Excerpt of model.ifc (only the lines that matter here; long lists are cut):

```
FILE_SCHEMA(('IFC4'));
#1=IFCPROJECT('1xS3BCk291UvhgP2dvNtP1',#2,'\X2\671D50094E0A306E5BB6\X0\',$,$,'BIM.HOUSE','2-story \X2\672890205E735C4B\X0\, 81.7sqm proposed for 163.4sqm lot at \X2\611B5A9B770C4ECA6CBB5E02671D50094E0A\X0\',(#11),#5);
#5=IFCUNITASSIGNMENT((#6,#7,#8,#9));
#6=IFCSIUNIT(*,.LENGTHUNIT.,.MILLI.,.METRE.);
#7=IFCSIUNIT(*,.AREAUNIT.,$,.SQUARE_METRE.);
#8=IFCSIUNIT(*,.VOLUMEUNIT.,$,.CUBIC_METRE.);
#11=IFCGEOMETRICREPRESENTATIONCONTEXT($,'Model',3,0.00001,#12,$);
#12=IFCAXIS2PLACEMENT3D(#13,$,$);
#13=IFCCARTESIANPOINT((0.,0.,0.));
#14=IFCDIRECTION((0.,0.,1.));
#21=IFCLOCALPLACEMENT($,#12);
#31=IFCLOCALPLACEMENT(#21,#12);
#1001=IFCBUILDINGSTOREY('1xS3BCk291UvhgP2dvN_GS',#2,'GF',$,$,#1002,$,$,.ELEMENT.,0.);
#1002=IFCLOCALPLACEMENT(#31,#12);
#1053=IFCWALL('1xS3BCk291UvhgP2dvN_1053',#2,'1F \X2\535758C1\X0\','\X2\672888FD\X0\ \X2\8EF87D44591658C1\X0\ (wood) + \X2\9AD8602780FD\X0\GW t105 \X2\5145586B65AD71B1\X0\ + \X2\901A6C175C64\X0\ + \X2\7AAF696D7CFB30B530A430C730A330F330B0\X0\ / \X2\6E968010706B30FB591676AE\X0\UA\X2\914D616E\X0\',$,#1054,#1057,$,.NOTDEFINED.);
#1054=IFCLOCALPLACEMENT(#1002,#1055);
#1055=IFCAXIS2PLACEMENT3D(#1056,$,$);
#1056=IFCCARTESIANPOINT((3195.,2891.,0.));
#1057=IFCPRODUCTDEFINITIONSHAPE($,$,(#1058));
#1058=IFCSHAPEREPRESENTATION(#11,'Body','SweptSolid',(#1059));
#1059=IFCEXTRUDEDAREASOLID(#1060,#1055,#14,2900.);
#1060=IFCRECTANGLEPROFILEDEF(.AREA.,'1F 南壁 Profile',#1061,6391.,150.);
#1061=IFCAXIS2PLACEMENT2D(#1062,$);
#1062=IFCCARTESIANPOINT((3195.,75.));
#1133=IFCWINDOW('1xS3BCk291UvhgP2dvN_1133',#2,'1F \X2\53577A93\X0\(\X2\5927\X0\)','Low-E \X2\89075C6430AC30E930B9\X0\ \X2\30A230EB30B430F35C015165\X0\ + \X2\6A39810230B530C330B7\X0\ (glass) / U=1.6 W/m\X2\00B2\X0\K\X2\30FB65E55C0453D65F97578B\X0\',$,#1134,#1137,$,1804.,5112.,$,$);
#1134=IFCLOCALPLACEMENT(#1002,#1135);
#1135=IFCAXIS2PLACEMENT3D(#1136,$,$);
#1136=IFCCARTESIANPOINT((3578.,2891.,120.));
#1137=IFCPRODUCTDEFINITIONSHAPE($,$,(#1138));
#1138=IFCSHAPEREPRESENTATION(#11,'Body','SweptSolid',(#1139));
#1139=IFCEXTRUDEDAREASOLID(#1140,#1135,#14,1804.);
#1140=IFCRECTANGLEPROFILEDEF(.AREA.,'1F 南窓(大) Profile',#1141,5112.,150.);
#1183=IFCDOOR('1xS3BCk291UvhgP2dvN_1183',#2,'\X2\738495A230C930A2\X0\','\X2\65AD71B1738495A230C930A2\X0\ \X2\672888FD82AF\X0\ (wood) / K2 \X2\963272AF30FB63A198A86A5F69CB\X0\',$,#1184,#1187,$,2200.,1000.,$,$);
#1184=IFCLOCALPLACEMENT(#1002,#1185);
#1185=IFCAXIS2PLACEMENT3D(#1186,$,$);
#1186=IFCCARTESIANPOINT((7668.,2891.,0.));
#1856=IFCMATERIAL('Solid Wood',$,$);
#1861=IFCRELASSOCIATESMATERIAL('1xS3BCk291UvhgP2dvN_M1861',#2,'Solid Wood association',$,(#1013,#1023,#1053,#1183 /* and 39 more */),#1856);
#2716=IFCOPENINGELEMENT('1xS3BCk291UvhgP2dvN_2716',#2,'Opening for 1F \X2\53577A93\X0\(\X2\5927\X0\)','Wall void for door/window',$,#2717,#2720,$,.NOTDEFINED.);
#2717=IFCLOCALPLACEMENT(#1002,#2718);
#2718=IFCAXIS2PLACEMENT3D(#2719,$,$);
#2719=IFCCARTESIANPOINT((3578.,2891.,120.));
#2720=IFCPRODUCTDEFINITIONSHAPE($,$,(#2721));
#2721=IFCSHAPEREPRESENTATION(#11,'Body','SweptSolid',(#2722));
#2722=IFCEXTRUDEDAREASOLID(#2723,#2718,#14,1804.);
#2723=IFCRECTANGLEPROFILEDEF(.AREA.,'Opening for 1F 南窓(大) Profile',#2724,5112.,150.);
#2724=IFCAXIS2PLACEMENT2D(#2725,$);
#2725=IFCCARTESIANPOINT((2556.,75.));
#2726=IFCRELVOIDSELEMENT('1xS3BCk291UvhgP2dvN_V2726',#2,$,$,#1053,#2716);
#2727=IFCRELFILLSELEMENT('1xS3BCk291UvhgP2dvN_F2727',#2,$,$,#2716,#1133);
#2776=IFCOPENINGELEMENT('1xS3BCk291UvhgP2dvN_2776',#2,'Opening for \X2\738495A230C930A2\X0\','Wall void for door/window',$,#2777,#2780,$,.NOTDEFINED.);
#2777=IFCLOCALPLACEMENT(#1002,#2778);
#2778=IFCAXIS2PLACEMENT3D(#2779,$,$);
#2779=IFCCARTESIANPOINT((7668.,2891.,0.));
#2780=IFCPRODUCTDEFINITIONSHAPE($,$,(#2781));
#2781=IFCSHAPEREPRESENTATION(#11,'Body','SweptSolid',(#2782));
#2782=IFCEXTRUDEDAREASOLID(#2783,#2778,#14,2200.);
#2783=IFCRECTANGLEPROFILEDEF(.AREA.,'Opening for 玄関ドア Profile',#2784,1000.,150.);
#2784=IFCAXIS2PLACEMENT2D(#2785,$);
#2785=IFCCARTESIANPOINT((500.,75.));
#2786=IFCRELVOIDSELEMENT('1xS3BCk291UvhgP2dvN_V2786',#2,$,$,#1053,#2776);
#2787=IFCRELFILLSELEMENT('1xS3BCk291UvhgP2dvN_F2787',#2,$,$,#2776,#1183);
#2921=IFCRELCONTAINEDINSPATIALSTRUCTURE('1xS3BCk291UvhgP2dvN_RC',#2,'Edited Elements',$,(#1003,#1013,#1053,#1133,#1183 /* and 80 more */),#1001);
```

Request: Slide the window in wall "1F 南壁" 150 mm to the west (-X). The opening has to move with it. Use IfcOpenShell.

```python
import ifcopenshell
import ifcopenshell.api.geometry
import ifcopenshell.util.placement
import ifcopenshell.util.unit

model = ifcopenshell.open("model.ifc")
unit_scale = ifcopenshell.util.unit.calculate_unit_scale(model)

window = model.by_guid("1xS3BCk291UvhgP2dvN_1133")
opening = window.FillsVoids[0].RelatingOpeningElement
wall = opening.VoidsElements[0].RelatingBuildingElement

wall_matrix = ifcopenshell.util.placement.get_local_placement(wall.ObjectPlacement)
shift = wall_matrix[:3, 0] * -0.15 / unit_scale
before = ifcopenshell.util.placement.get_local_placement(window.ObjectPlacement)[:3, 3].copy()

# The window is not placed relative to its opening, so move both.
for product in (opening, window):
    matrix = ifcopenshell.util.placement.get_local_placement(product.ObjectPlacement)
    matrix[:3, 3] += shift
    ifcopenshell.api.geometry.edit_object_placement(model, product=product, matrix=matrix, is_si=False)

after = ifcopenshell.util.placement.get_local_placement(window.ObjectPlacement)[:3, 3]
print("window moved by", (after - before).round(3) + 0.0)

model.write("model_edited.ifc")
```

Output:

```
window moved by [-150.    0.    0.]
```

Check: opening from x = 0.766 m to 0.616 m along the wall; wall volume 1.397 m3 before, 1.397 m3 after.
